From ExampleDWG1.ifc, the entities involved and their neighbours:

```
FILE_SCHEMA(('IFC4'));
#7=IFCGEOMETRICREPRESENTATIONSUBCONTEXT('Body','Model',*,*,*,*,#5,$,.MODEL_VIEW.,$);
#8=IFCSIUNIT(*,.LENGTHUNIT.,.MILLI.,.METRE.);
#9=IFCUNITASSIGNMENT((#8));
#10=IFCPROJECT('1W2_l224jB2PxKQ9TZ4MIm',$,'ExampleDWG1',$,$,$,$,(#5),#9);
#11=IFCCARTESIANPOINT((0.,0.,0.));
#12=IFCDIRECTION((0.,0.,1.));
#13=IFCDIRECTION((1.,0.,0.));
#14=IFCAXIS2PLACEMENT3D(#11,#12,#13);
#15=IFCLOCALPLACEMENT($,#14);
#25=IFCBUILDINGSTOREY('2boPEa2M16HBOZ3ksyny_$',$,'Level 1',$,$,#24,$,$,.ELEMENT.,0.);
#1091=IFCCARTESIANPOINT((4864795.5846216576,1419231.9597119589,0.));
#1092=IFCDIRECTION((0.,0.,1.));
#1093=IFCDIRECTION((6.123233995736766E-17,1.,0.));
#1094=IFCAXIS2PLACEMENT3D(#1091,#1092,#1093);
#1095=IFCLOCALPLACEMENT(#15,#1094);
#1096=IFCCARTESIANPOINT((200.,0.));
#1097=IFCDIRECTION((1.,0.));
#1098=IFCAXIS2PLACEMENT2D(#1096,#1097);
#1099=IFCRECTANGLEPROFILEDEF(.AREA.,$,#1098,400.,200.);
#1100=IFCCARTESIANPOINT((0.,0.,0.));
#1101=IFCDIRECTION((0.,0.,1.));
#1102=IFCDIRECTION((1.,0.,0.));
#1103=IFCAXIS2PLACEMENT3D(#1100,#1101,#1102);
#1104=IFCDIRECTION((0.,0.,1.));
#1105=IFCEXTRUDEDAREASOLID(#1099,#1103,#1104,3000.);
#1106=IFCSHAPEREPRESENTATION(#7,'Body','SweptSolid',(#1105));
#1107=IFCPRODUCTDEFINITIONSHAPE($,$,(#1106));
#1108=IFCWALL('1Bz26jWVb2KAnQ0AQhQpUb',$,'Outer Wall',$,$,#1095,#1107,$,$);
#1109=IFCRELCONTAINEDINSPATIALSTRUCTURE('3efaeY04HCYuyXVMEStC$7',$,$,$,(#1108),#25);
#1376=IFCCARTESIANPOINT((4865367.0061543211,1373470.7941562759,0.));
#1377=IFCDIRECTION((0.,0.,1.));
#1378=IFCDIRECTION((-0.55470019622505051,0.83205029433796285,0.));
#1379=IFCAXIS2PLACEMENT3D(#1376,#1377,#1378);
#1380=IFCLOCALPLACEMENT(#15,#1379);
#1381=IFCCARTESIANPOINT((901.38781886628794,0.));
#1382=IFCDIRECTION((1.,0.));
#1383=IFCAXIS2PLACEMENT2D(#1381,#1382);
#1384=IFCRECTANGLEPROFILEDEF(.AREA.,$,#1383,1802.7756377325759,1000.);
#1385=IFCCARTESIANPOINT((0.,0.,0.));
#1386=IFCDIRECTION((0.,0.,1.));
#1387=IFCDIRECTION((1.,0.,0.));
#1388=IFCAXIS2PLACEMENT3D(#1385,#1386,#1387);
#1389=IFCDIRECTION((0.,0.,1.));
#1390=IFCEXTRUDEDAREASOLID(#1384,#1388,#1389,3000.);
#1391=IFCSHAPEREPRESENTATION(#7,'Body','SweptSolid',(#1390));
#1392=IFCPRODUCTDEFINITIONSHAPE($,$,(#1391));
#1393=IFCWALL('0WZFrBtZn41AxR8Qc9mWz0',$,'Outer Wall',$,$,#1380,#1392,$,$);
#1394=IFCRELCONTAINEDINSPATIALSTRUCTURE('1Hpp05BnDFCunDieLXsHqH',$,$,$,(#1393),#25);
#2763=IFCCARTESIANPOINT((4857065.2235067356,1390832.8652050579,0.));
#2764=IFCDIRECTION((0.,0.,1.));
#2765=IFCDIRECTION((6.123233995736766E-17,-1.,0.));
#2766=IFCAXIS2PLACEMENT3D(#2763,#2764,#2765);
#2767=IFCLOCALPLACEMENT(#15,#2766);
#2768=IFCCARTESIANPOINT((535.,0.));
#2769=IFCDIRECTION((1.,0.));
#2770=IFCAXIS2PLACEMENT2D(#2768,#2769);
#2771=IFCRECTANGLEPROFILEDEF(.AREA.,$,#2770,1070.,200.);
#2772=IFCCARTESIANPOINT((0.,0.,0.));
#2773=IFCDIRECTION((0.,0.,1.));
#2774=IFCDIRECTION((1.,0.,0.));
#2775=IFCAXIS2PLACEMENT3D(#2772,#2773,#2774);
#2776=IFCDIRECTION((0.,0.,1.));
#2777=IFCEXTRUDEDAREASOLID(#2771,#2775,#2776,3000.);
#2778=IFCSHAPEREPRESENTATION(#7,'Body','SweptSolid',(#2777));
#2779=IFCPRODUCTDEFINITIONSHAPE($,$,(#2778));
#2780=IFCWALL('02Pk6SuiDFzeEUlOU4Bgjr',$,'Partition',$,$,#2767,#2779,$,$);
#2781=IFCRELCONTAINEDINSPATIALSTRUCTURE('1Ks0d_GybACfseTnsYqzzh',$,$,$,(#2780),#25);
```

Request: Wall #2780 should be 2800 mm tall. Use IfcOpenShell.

```python
import ifcopenshell
import ifcopenshell.geom
import ifcopenshell.util.representation
import ifcopenshell.util.shape
import ifcopenshell.util.unit

model = ifcopenshell.open("ExampleDWG1.ifc")
unit_scale = ifcopenshell.util.unit.calculate_unit_scale(model)
settings = ifcopenshell.geom.settings()


def volume(element):
    """Net volume in cubic metres, openings subtracted."""
    shape = ifcopenshell.geom.create_shape(settings, element)
    return ifcopenshell.util.shape.get_volume(shape.geometry)


wall = model.by_guid("02Pk6SuiDFzeEUlOU4Bgjr")
before = volume(wall)

body = ifcopenshell.util.representation.get_representation(wall, "Model", "Body")
solid = body.Items[0]
old_height = solid.Depth
solid.Depth = 2.8 / unit_scale
after = volume(wall)

print(f"height {old_height:g} -> {solid.Depth:g}, volume {before:.3f} -> {after:.3f} m3")

model.write("ExampleDWG1_updated.ifc")
```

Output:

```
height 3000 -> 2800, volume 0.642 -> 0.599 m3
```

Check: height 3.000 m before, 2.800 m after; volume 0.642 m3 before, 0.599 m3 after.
